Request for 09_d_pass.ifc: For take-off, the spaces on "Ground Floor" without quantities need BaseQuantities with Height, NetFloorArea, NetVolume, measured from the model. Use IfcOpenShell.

First a look at what the model holds.

```python
import ifcopenshell
import ifcopenshell.util.element
import ifcopenshell.util.unit

model = ifcopenshell.open("09_d_pass.ifc")
print(model.schema)
for unit_type in ("LENGTHUNIT", "AREAUNIT", "VOLUMEUNIT"):
    print(unit_type, ifcopenshell.util.unit.calculate_unit_scale(model, unit_type))
storey = next(s for s in model.by_type("IfcBuildingStorey") if s.Name == "Ground Floor")
spaces = [e for e in ifcopenshell.util.element.get_decomposition(storey) if e.is_a("IfcSpace")]
for e in sorted(spaces, key=lambda e: e.id()):
    print(e.id(), e.is_a(), e.Name, list(ifcopenshell.util.element.get_psets(e, qtos_only=True)), sep=" | ")
```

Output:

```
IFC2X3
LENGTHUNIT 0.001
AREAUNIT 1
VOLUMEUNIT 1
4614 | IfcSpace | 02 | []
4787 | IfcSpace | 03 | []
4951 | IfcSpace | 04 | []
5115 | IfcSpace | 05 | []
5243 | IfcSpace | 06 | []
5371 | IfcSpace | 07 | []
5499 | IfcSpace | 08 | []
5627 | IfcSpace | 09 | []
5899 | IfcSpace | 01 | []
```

```python
import ifcopenshell
import ifcopenshell.api.pset
import ifcopenshell.geom
import ifcopenshell.util.element
import ifcopenshell.util.shape
import ifcopenshell.util.unit

model = ifcopenshell.open("09_d_pass.ifc")
unit_scale = ifcopenshell.util.unit.calculate_unit_scale(model)
area_scale = ifcopenshell.util.unit.calculate_unit_scale(model, "AREAUNIT")
volume_scale = ifcopenshell.util.unit.calculate_unit_scale(model, "VOLUMEUNIT")
settings = ifcopenshell.geom.settings()

storey = next(s for s in model.by_type("IfcBuildingStorey") if s.Name == "Ground Floor")
spaces = [e for e in ifcopenshell.util.element.get_decomposition(storey) if e.is_a("IfcSpace")]

for e in sorted(spaces, key=lambda e: e.id()):
    if ifcopenshell.util.element.get_psets(e, qtos_only=True, should_inherit=False):
        continue
    # Geometry comes back in metres, in the element's own axes.
    shape = ifcopenshell.geom.create_shape(settings, e)
    values = {
        "Height": ifcopenshell.util.shape.get_z(shape.geometry) / unit_scale,
        "NetFloorArea": ifcopenshell.util.shape.get_footprint_area(shape.geometry) / area_scale,
        "NetVolume": ifcopenshell.util.shape.get_volume(shape.geometry) / volume_scale,
    }
    qto = ifcopenshell.api.pset.add_qto(model, product=e, name="BaseQuantities")
    ifcopenshell.api.pset.edit_qto(model, qto=qto, properties=values)
    print(e.id(), {k: round(v, 3) for k, v in values.items()})

model.write("09_d_pass_v2.ifc")
```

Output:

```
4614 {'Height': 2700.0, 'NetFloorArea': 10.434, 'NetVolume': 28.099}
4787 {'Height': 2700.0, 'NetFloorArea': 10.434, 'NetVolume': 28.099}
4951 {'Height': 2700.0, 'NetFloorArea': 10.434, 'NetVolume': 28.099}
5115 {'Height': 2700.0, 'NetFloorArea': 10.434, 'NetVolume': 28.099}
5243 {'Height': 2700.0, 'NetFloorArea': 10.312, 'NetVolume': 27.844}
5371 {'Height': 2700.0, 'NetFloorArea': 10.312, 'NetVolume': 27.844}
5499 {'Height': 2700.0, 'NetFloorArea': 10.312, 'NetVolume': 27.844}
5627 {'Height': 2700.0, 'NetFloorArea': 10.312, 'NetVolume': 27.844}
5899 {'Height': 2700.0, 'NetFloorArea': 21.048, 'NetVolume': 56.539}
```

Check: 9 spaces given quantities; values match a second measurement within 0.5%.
